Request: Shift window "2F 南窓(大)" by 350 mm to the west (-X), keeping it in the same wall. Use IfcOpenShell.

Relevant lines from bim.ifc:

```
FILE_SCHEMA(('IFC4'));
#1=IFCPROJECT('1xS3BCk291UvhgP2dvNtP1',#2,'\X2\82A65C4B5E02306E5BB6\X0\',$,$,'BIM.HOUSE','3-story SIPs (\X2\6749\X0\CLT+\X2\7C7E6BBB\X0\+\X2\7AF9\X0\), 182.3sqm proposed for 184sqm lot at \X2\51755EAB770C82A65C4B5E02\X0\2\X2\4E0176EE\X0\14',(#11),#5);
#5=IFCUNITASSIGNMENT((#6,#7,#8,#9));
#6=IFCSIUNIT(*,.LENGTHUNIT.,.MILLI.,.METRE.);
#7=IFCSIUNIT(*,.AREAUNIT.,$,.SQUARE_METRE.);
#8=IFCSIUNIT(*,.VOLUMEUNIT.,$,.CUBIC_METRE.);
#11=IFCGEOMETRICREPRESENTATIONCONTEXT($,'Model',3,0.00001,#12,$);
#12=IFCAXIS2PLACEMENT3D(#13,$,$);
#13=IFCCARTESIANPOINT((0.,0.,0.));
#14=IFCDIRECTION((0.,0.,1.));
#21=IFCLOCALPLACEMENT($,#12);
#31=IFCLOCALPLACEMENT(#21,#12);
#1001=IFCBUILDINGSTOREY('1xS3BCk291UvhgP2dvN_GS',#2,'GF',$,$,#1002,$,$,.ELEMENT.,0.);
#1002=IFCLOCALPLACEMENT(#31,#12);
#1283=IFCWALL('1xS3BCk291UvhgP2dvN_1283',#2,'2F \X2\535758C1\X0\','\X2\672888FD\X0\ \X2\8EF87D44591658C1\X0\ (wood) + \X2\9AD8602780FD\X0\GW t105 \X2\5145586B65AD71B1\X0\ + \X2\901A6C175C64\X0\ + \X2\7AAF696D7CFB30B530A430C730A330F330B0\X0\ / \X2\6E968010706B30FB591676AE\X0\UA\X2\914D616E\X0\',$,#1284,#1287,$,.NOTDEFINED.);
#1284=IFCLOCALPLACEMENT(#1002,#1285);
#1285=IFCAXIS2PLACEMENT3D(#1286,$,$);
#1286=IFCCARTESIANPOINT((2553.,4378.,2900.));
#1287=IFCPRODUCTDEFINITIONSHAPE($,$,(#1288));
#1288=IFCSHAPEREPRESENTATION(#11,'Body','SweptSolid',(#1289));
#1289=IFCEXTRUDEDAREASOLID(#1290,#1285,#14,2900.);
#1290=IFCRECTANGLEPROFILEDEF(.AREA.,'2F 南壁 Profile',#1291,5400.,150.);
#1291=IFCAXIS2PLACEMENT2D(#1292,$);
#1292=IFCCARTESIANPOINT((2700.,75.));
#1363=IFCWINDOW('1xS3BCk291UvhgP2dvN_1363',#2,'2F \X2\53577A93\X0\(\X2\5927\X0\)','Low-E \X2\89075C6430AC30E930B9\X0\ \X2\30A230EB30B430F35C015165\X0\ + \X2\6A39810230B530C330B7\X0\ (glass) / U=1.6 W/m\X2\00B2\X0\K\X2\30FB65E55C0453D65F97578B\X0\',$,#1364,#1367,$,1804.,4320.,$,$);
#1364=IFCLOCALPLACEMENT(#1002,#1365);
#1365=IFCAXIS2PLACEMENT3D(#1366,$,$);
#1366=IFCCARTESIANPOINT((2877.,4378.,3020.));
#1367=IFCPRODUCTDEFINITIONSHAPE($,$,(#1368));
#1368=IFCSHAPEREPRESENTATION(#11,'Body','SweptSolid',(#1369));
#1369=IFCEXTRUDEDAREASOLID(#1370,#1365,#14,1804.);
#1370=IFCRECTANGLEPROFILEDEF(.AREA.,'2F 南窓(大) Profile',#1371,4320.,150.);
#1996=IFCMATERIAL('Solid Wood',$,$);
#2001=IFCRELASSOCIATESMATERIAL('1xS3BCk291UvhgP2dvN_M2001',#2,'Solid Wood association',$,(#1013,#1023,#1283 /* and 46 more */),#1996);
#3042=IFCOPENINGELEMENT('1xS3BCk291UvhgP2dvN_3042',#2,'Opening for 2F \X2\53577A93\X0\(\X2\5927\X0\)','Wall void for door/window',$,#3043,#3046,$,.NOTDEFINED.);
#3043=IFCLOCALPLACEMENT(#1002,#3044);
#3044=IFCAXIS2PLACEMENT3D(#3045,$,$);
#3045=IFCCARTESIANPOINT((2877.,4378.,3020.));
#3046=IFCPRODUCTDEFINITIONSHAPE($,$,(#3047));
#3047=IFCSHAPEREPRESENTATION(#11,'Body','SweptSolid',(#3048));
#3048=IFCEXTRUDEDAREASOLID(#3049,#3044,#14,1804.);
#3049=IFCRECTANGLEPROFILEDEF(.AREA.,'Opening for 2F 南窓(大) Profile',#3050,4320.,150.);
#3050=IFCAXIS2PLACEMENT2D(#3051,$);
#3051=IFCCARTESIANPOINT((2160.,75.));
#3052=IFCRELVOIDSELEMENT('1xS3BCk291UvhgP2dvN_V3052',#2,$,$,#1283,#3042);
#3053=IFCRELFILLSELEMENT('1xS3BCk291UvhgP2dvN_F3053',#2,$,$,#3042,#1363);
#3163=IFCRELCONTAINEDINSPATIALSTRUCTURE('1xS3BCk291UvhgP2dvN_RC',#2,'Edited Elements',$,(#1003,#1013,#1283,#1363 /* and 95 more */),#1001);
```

```python
import ifcopenshell
import ifcopenshell.api.geometry
import ifcopenshell.util.placement

model = ifcopenshell.open("bim.ifc")

window = model.by_guid("1xS3BCk291UvhgP2dvN_1363")
opening = window.FillsVoids[0].RelatingOpeningElement
wall = opening.VoidsElements[0].RelatingBuildingElement

wall_matrix = ifcopenshell.util.placement.get_local_placement(wall.ObjectPlacement)
shift = wall_matrix[:3, 0] * -350.0
before = ifcopenshell.util.placement.get_local_placement(window.ObjectPlacement)[:3, 3].copy()

# The window is not placed relative to its opening, so move both.
for product in (opening, window):
    matrix = ifcopenshell.util.placement.get_local_placement(product.ObjectPlacement)
    matrix[:3, 3] += shift
    ifcopenshell.api.geometry.edit_object_placement(model, product=product, matrix=matrix, is_si=False)

after = ifcopenshell.util.placement.get_local_placement(window.ObjectPlacement)[:3, 3]
print("window moved by", (after - before).round(3) + 0.0)

model.write("bim-out.ifc")
```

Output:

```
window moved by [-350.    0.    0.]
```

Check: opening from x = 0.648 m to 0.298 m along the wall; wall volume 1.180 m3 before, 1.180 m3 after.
